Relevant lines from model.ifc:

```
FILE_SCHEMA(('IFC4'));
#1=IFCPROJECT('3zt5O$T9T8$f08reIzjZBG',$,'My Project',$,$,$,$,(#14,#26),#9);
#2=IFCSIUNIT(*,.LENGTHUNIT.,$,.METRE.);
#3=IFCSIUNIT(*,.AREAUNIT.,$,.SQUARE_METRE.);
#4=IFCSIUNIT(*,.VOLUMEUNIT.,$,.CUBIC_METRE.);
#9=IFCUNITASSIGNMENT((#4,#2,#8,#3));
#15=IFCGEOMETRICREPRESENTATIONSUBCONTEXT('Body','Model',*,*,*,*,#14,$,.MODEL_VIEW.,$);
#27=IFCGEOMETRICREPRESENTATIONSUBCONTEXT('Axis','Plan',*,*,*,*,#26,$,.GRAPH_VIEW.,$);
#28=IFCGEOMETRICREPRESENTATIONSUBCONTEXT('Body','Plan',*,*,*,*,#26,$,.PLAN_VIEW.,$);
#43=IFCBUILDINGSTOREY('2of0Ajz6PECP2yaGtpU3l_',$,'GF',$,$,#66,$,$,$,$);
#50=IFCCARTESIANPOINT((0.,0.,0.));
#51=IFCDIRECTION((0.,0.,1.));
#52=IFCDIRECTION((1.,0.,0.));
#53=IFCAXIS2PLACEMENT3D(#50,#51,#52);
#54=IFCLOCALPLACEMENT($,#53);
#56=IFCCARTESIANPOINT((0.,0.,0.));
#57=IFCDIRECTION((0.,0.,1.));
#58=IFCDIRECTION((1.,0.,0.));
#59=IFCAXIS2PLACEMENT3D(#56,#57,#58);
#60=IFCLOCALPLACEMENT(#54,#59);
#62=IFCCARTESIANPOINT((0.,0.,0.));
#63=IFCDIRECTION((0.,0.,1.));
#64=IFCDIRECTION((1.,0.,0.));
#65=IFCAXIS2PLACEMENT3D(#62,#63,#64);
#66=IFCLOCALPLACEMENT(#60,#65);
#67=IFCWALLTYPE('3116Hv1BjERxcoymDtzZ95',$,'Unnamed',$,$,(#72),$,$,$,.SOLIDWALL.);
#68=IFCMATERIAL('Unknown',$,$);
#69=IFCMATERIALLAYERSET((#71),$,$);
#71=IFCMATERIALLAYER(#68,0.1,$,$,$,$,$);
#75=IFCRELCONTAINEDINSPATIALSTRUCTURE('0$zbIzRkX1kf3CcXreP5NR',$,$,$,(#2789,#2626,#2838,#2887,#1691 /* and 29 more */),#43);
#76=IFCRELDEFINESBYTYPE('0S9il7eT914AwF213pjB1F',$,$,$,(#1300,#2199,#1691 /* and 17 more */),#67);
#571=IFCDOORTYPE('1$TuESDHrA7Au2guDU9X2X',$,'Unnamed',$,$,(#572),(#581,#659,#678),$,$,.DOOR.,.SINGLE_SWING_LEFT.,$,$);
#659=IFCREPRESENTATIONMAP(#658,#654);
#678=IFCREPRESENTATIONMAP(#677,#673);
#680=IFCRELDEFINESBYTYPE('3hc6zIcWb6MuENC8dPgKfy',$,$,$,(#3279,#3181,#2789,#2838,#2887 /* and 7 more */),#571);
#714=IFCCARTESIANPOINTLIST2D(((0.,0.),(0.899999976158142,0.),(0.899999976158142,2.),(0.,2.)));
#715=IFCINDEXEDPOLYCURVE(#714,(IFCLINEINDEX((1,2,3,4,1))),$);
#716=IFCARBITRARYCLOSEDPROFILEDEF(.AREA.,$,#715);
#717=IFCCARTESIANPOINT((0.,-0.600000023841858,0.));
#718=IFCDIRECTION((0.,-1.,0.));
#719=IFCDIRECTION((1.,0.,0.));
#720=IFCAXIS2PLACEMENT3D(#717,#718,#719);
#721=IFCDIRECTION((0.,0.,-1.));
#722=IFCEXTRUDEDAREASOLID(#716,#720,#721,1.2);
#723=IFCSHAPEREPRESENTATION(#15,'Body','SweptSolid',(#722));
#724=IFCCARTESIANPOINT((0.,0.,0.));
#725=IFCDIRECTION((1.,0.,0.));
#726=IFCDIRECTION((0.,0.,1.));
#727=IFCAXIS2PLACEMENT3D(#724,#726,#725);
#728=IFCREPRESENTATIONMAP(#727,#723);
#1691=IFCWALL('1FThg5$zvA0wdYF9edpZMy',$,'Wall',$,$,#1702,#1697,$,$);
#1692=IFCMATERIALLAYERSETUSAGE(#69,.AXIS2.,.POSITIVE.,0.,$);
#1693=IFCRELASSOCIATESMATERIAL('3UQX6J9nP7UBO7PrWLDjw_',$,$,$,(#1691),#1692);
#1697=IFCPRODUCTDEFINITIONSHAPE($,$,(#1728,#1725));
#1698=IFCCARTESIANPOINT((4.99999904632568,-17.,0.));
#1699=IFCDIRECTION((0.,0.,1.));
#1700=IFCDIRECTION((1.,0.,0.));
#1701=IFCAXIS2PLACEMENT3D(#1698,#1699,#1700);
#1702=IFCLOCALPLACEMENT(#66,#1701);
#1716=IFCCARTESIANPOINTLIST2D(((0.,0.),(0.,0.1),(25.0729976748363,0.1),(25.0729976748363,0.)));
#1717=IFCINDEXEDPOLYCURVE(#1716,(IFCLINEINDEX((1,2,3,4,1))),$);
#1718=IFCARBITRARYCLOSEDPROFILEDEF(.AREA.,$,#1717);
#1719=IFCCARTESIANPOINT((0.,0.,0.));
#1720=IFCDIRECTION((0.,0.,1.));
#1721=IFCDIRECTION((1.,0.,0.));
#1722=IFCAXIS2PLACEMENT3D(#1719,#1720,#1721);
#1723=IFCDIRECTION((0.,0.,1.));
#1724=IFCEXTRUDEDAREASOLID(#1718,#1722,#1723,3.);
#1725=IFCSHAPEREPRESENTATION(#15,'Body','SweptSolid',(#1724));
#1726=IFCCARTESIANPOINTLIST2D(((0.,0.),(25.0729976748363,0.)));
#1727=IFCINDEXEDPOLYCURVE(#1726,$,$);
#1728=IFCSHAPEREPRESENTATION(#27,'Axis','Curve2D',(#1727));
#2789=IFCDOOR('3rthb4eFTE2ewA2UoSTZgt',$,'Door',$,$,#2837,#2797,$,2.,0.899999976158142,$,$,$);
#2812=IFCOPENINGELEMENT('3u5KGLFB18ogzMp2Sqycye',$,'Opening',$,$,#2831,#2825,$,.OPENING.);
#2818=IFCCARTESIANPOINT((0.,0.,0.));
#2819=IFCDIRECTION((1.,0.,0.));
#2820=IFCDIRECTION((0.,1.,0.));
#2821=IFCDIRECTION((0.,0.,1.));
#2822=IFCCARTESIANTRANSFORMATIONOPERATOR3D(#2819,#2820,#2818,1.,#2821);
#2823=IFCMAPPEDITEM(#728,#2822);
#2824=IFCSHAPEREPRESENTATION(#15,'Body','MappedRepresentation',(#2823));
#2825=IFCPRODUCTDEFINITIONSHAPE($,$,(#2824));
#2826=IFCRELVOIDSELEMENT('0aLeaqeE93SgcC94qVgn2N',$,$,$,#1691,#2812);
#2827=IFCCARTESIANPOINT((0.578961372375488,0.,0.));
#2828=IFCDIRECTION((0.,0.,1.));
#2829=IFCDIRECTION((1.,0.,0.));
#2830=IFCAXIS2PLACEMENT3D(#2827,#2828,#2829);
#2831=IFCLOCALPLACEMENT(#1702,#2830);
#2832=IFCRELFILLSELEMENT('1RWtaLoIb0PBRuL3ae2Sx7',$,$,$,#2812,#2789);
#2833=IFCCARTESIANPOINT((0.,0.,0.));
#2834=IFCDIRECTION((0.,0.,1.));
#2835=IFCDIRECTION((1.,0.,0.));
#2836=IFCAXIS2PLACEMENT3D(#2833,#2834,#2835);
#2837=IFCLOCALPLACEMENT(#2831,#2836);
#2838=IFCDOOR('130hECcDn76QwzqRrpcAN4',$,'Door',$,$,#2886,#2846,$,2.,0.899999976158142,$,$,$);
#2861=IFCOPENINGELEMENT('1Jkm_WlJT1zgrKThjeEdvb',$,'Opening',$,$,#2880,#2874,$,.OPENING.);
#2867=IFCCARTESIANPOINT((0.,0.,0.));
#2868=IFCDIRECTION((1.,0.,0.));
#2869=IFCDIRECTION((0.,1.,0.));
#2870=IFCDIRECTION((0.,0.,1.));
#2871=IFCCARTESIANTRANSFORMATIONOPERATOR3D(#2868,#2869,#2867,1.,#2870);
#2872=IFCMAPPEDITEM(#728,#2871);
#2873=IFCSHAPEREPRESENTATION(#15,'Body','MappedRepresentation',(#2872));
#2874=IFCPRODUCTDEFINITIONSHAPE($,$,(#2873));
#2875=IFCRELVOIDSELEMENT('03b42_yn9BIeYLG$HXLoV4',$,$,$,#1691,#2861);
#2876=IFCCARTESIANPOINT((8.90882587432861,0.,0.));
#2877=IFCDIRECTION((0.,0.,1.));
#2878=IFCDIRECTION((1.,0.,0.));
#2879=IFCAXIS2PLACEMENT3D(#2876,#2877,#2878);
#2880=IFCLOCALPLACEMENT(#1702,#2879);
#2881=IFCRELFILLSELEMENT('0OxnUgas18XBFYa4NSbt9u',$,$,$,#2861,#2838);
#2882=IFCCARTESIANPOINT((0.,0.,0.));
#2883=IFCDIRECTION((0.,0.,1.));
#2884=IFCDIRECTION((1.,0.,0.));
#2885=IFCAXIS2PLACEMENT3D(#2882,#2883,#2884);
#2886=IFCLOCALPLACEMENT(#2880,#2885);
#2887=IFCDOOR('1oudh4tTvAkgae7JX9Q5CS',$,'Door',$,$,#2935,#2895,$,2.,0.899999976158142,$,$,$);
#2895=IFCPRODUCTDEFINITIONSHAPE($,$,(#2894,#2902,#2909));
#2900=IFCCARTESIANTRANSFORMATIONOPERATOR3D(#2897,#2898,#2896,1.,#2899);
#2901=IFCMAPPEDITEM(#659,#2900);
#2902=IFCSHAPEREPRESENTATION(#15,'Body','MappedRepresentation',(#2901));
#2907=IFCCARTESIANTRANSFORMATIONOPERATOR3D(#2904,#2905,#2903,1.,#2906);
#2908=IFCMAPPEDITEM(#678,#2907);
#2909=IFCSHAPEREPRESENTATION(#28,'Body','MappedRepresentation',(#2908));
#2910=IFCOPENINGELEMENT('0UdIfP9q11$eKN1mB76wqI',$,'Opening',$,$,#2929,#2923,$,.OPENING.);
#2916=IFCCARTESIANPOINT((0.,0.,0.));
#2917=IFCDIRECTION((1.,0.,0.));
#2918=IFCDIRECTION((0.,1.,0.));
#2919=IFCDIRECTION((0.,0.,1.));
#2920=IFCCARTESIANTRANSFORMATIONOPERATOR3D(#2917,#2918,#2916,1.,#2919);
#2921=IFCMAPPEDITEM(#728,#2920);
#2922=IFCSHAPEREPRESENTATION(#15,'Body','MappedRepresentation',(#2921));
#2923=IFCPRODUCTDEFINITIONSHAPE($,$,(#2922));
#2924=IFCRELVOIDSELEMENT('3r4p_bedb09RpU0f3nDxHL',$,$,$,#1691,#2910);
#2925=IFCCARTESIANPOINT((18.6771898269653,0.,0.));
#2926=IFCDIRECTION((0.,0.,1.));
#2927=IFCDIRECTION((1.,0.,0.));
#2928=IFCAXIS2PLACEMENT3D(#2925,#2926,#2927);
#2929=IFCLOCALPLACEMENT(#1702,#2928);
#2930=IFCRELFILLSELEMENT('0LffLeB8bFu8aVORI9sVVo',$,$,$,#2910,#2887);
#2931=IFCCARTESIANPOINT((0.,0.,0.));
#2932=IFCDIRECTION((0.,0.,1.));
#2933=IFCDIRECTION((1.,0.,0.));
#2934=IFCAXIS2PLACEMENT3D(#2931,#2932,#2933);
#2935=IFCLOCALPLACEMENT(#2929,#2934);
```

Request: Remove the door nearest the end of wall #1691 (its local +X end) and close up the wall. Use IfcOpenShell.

```python
import ifcopenshell
import ifcopenshell.api.feature
import ifcopenshell.api.root
import ifcopenshell.geom
import ifcopenshell.util.shape

model = ifcopenshell.open("model.ifc")
settings = ifcopenshell.geom.settings()


def volume(element):
    """Net volume in cubic metres, openings subtracted."""
    shape = ifcopenshell.geom.create_shape(settings, element)
    return ifcopenshell.util.shape.get_volume(shape.geometry)


door = model.by_guid("1oudh4tTvAkgae7JX9Q5CS")
opening = door.FillsVoids[0].RelatingOpeningElement
wall = opening.VoidsElements[0].RelatingBuildingElement
before = volume(wall)

ifcopenshell.api.root.remove_product(model, product=door)
ifcopenshell.api.feature.remove_feature(model, feature=opening)

after = volume(wall)

print(f"wall volume {before:.3f} -> {after:.3f} m3")

model.write("model_edited.ifc")
```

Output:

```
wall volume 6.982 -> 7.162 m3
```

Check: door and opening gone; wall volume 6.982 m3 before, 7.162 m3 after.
